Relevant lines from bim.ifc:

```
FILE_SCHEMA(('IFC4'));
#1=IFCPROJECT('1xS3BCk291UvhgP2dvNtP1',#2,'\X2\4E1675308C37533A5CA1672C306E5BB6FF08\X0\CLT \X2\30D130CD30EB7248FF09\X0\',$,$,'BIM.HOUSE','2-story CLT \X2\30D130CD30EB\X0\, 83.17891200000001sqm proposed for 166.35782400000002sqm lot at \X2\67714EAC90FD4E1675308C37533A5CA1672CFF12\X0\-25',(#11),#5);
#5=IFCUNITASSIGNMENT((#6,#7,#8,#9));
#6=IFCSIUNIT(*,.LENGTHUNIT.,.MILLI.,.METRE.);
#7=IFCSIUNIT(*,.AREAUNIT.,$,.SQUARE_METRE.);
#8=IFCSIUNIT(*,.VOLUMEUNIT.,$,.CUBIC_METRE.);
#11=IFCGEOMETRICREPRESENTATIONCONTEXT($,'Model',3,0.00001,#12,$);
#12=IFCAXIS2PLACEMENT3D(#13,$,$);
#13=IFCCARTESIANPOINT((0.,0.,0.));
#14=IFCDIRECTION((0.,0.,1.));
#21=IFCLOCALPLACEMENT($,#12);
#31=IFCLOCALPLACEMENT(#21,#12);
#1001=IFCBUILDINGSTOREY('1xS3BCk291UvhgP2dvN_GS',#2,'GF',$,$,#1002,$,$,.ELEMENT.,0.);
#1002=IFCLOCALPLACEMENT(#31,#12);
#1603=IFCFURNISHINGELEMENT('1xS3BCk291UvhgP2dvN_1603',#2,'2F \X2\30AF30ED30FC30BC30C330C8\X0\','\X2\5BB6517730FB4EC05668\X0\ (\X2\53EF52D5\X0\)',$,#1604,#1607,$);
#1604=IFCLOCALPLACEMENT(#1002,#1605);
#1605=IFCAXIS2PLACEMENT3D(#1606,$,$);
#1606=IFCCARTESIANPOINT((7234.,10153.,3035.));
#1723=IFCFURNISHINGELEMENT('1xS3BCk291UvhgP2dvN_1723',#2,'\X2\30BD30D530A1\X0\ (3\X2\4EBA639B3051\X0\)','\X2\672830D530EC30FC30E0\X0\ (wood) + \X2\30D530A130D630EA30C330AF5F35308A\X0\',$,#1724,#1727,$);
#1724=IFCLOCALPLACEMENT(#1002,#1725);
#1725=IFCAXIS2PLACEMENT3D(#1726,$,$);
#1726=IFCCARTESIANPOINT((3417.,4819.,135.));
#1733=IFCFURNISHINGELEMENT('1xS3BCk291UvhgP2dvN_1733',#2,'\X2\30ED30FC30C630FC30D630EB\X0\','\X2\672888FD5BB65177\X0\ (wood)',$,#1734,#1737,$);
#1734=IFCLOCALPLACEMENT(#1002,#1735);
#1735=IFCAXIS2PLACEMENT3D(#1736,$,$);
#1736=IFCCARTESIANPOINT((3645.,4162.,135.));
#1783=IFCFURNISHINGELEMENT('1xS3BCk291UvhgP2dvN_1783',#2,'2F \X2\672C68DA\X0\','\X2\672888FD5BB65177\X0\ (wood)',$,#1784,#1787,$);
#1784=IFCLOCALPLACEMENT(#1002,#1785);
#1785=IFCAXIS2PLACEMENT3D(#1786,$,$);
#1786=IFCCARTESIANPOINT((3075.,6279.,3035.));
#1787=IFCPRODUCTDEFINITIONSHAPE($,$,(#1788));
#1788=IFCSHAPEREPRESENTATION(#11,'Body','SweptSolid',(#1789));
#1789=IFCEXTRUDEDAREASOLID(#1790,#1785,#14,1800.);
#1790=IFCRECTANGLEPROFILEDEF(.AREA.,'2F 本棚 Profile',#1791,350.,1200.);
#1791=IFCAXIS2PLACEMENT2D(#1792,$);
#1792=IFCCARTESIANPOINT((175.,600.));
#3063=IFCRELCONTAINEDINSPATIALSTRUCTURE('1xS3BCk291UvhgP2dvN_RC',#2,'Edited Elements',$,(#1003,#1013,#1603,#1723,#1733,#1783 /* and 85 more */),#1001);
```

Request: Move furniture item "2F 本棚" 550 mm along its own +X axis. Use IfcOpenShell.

```python
import ifcopenshell
import ifcopenshell.api.geometry
import ifcopenshell.util.placement
import ifcopenshell.util.unit

model = ifcopenshell.open("bim.ifc")
unit_scale = ifcopenshell.util.unit.calculate_unit_scale(model)

item = model.by_id(1783)
matrix = ifcopenshell.util.placement.get_local_placement(item.ObjectPlacement)
matrix[:3, 3] += matrix[:3, 0] * 0.55 / unit_scale
ifcopenshell.api.geometry.edit_object_placement(model, product=item, matrix=matrix, is_si=False)

print(ifcopenshell.util.placement.get_local_placement(item.ObjectPlacement).round(3) + 0.0)

model.write("bim_v2.ifc")
```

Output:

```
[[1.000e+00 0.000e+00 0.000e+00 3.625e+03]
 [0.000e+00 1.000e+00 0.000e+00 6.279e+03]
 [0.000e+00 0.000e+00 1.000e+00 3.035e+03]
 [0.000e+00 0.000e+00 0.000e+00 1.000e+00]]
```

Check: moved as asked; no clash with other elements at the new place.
